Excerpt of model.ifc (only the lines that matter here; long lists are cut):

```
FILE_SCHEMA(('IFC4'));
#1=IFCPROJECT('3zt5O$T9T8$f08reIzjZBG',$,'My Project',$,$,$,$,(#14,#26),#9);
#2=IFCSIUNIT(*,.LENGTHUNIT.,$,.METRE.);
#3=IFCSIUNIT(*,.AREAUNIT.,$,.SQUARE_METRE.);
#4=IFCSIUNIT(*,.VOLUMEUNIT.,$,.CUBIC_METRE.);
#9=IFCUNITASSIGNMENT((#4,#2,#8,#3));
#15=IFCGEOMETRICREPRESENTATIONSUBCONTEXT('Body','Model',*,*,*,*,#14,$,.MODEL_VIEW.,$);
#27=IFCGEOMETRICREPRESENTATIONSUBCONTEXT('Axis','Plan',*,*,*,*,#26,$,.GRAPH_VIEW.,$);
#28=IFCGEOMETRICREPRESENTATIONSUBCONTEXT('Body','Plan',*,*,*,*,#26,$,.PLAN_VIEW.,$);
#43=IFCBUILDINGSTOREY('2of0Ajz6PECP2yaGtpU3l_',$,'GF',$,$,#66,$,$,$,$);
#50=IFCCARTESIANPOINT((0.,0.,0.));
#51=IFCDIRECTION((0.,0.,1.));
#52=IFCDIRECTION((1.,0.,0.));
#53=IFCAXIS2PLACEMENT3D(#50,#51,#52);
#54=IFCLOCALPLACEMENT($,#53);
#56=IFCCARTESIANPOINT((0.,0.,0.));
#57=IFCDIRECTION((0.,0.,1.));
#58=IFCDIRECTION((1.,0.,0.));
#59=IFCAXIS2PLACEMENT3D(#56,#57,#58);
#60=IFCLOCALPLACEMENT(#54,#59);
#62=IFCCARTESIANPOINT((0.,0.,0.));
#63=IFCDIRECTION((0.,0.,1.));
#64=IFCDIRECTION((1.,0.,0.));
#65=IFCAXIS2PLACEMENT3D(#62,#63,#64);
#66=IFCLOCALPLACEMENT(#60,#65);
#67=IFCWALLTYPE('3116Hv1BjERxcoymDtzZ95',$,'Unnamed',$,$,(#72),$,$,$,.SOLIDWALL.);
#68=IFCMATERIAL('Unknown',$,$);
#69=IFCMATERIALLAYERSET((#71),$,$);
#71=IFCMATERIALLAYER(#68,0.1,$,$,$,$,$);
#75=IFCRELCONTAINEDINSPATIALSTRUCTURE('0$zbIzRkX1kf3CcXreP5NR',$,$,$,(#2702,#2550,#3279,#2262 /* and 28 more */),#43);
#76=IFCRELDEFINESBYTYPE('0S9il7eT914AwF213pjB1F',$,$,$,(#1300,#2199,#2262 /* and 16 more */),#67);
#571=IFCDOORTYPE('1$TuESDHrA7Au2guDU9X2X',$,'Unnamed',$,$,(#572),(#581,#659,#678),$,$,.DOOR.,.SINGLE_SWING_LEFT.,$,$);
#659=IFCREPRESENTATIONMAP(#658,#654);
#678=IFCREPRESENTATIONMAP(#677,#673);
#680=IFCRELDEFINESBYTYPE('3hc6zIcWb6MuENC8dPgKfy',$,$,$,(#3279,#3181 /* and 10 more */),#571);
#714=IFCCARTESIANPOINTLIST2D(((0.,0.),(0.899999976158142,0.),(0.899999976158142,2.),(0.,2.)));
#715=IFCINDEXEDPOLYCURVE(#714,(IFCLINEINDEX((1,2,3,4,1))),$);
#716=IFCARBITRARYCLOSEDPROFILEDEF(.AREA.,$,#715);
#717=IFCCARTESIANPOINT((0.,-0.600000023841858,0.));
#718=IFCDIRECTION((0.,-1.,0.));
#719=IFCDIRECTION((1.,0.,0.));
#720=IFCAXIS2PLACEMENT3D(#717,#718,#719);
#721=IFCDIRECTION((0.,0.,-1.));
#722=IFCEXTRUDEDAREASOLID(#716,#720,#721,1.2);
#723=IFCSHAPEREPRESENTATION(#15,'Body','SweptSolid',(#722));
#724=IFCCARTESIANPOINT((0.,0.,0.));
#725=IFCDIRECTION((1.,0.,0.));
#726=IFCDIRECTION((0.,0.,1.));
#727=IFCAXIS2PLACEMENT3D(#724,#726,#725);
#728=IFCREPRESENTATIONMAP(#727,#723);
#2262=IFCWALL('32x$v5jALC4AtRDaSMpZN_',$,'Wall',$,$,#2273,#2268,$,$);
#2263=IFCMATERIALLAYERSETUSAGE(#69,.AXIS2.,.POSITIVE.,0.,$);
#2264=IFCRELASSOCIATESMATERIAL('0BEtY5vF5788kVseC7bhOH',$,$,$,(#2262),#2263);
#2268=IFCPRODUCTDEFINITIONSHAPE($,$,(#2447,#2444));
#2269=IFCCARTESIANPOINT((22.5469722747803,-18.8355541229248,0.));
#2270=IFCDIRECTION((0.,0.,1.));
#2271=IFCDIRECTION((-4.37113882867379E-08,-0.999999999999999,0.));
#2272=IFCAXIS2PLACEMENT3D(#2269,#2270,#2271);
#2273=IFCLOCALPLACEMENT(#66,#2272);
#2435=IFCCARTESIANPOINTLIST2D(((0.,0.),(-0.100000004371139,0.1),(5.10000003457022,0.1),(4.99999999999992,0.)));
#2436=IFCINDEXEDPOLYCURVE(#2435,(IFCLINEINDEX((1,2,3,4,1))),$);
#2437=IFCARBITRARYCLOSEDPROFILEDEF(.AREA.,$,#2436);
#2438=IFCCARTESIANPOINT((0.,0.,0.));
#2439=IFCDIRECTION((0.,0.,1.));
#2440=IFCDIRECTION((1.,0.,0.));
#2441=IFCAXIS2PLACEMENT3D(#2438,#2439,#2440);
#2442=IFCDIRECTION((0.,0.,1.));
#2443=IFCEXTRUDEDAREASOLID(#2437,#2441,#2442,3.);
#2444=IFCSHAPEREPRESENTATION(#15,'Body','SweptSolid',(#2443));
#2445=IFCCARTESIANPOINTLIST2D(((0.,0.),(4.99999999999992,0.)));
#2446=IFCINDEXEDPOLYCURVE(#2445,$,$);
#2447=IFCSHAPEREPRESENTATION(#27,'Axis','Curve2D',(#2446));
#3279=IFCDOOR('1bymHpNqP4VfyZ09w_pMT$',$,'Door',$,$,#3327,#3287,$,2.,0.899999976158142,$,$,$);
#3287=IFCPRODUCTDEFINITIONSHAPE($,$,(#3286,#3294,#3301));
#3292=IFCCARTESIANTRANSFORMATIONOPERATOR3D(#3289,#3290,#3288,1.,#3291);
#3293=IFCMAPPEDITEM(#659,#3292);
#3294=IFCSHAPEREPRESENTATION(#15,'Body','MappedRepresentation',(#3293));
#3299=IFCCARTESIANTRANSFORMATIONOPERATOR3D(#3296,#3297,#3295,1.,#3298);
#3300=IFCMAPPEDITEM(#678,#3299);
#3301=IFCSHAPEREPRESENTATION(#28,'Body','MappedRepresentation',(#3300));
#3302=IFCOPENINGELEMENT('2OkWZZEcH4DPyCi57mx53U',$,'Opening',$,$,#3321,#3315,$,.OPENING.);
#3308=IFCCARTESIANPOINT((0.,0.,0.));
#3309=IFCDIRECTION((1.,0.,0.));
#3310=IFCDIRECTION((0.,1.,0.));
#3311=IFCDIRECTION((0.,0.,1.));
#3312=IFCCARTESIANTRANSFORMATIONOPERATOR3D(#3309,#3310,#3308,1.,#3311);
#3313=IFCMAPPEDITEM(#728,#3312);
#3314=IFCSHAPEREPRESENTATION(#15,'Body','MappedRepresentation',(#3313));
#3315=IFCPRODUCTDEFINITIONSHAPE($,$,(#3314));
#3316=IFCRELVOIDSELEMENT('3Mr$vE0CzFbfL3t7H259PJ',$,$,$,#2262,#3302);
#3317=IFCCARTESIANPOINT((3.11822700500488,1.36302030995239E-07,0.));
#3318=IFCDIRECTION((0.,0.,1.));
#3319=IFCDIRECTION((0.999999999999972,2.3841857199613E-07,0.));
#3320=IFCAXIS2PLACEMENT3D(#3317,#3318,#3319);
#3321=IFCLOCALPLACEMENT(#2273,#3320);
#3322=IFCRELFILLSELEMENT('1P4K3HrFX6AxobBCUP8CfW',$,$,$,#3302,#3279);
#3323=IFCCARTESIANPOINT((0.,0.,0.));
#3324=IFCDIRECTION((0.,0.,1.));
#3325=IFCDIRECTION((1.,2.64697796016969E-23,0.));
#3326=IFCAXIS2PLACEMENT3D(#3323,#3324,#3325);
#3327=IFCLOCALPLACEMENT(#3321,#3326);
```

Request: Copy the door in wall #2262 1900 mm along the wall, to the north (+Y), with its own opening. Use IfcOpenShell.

```python
import ifcopenshell
import ifcopenshell.api.feature
import ifcopenshell.api.geometry
import ifcopenshell.api.root
import ifcopenshell.geom
import ifcopenshell.util.element
import ifcopenshell.util.placement
import ifcopenshell.util.shape

model = ifcopenshell.open("model.ifc")
settings = ifcopenshell.geom.settings()


def volume(element):
    """Net volume in cubic metres, openings subtracted."""
    shape = ifcopenshell.geom.create_shape(settings, element)
    return ifcopenshell.util.shape.get_volume(shape.geometry)


door = model.by_guid("1bymHpNqP4VfyZ09w_pMT$")
opening = door.FillsVoids[0].RelatingOpeningElement
wall = opening.VoidsElements[0].RelatingBuildingElement
before = volume(wall)
shift = ifcopenshell.util.placement.get_local_placement(wall.ObjectPlacement)[:3, 0] * -1.9

# copy_class copies the void relationship, type, container and properties, but no geometry.
new_opening = ifcopenshell.api.root.copy_class(model, product=opening)
new_opening.Representation = ifcopenshell.util.element.copy_deep(
    model, opening.Representation, exclude=["IfcGeometricRepresentationContext", "IfcRepresentationMap"]
)
new_door = ifcopenshell.api.root.copy_class(model, product=door)
new_door.Representation = ifcopenshell.util.element.copy_deep(
    model, door.Representation, exclude=["IfcGeometricRepresentationContext", "IfcRepresentationMap"]
)
ifcopenshell.api.feature.add_filling(model, opening=new_opening, element=new_door)

for old, new in ((opening, new_opening), (door, new_door)):
    matrix = ifcopenshell.util.placement.get_local_placement(old.ObjectPlacement)
    matrix[:3, 3] += shift
    ifcopenshell.api.geometry.edit_object_placement(model, product=new, matrix=matrix, is_si=False)

after = volume(wall)

print(f"wall volume {before:.3f} -> {after:.3f} m3")

model.write("model_updated.ifc")
```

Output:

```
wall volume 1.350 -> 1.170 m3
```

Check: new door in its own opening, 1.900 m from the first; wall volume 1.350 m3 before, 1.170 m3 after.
